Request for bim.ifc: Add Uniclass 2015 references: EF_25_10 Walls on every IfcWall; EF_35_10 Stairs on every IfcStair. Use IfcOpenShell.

First a look at what the model holds.

```python
import ifcopenshell

model = ifcopenshell.open("bim.ifc")
print(model.schema)
print("classifications:", [c.Name for c in model.by_type("IfcClassification")])
for ifc_class in ("IfcDoor", "IfcRoof", "IfcStair", "IfcWall", "IfcWindow"):
    print(ifc_class, len(model.by_type(ifc_class)))
```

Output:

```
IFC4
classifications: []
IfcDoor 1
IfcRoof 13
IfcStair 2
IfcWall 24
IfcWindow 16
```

```python
import ifcopenshell
import ifcopenshell.api.classification

model = ifcopenshell.open("bim.ifc")

system = ifcopenshell.api.classification.add_classification(model, classification="Uniclass 2015")

codes = {
    "IfcWall": ("EF_25_10", "Walls"),
    "IfcStair": ("EF_35_10", "Stairs"),
}
for ifc_class, (code, name) in codes.items():
    products = model.by_type(ifc_class)
    ifcopenshell.api.classification.add_reference(
        model, products=products, classification=system, identification=code, name=name
    )
    print(code, len(products))

model.write("bim_updated.ifc")
```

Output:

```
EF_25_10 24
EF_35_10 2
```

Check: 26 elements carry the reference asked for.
